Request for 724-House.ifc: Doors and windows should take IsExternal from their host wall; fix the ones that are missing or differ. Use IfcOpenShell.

First a look at what the model holds.

```python
import ifcopenshell
import ifcopenshell.util.element

model = ifcopenshell.open("724-House.ifc")
print(model.schema)
seen = {}
for e in model.by_type("IfcDoor") + model.by_type("IfcWindow"):
    if not e.FillsVoids:
        continue
    host = e.FillsVoids[0].RelatingOpeningElement.VoidsElements[0].RelatingBuildingElement
    own = ifcopenshell.util.element.get_pset(e, f"Pset_{e.is_a()[3:].removesuffix('StandardCase')}Common", "IsExternal")
    wall = ifcopenshell.util.element.get_pset(host, "Pset_WallCommon", "IsExternal")
    seen[e.is_a(), own, wall] = seen.get((e.is_a(), own, wall), 0) + 1
for (cls, own, wall), count in sorted(seen.items(), key=str):
    print(count, cls, "IsExternal:", own, "| host wall:", wall)
```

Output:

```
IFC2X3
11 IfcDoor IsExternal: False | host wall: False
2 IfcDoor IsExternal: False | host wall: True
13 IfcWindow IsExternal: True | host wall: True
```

```python
import ifcopenshell
import ifcopenshell.api.pset
import ifcopenshell.util.element

model = ifcopenshell.open("724-House.ifc")

count = 0
for ifc_class, pset_name in (("IfcDoor", "Pset_DoorCommon"), ("IfcWindow", "Pset_WindowCommon")):
    for e in model.by_type(ifc_class):
        if not e.FillsVoids:
            continue
        host = e.FillsVoids[0].RelatingOpeningElement.VoidsElements[0].RelatingBuildingElement
        external = ifcopenshell.util.element.get_pset(host, "Pset_WallCommon", "IsExternal")
        if external is None or ifcopenshell.util.element.get_pset(e, pset_name, "IsExternal") == external:
            continue
        pset = ifcopenshell.api.pset.add_pset(model, product=e, name=pset_name)
        ifcopenshell.api.pset.edit_pset(model, pset=pset, properties={"IsExternal": external})
        count += 1

print(count, "updated")

model.write("724-House_edited.ifc")
```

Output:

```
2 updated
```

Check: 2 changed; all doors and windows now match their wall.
